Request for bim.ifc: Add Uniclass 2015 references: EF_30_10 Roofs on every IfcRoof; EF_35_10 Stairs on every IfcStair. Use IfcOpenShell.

First a look at what the model holds.

```python
import ifcopenshell

model = ifcopenshell.open("bim.ifc")
print(model.schema)
print("classifications:", [c.Name for c in model.by_type("IfcClassification")])
for ifc_class in ("IfcDoor", "IfcRoof", "IfcStair", "IfcWall", "IfcWindow"):
    print(ifc_class, len(model.by_type(ifc_class)))
```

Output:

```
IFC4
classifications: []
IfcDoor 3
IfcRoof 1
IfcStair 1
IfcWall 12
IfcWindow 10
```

```python
import ifcopenshell
import ifcopenshell.api.classification

model = ifcopenshell.open("bim.ifc")

system = ifcopenshell.api.classification.add_classification(model, classification="Uniclass 2015")

codes = {
    "IfcRoof": ("EF_30_10", "Roofs"),
    "IfcStair": ("EF_35_10", "Stairs"),
}
for ifc_class, (code, name) in codes.items():
    products = model.by_type(ifc_class)
    ifcopenshell.api.classification.add_reference(
        model, products=products, classification=system, identification=code, name=name
    )
    print(code, len(products))

model.write("bim_rev.ifc")
```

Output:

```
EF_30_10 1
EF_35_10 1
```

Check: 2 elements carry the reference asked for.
